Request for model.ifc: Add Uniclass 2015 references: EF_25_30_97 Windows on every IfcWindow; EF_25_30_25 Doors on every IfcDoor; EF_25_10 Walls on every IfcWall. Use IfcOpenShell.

First a look at what the model holds.

```python
import ifcopenshell

model = ifcopenshell.open("model.ifc")
print(model.schema)
print("classifications:", [c.Name for c in model.by_type("IfcClassification")])
for ifc_class in ("IfcDoor", "IfcRoof", "IfcStair", "IfcWall", "IfcWindow"):
    print(ifc_class, len(model.by_type(ifc_class)))
```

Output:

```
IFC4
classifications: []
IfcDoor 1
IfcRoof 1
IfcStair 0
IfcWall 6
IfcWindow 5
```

```python
import ifcopenshell
import ifcopenshell.api.classification

model = ifcopenshell.open("model.ifc")

system = ifcopenshell.api.classification.add_classification(model, classification="Uniclass 2015")

codes = {
    "IfcWindow": ("EF_25_30_97", "Windows"),
    "IfcDoor": ("EF_25_30_25", "Doors"),
    "IfcWall": ("EF_25_10", "Walls"),
}
for ifc_class, (code, name) in codes.items():
    products = model.by_type(ifc_class)
    ifcopenshell.api.classification.add_reference(
        model, products=products, classification=system, identification=code, name=name
    )
    print(code, len(products))

model.write("model_updated.ifc")
```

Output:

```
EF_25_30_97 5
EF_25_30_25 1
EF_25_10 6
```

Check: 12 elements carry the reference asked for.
